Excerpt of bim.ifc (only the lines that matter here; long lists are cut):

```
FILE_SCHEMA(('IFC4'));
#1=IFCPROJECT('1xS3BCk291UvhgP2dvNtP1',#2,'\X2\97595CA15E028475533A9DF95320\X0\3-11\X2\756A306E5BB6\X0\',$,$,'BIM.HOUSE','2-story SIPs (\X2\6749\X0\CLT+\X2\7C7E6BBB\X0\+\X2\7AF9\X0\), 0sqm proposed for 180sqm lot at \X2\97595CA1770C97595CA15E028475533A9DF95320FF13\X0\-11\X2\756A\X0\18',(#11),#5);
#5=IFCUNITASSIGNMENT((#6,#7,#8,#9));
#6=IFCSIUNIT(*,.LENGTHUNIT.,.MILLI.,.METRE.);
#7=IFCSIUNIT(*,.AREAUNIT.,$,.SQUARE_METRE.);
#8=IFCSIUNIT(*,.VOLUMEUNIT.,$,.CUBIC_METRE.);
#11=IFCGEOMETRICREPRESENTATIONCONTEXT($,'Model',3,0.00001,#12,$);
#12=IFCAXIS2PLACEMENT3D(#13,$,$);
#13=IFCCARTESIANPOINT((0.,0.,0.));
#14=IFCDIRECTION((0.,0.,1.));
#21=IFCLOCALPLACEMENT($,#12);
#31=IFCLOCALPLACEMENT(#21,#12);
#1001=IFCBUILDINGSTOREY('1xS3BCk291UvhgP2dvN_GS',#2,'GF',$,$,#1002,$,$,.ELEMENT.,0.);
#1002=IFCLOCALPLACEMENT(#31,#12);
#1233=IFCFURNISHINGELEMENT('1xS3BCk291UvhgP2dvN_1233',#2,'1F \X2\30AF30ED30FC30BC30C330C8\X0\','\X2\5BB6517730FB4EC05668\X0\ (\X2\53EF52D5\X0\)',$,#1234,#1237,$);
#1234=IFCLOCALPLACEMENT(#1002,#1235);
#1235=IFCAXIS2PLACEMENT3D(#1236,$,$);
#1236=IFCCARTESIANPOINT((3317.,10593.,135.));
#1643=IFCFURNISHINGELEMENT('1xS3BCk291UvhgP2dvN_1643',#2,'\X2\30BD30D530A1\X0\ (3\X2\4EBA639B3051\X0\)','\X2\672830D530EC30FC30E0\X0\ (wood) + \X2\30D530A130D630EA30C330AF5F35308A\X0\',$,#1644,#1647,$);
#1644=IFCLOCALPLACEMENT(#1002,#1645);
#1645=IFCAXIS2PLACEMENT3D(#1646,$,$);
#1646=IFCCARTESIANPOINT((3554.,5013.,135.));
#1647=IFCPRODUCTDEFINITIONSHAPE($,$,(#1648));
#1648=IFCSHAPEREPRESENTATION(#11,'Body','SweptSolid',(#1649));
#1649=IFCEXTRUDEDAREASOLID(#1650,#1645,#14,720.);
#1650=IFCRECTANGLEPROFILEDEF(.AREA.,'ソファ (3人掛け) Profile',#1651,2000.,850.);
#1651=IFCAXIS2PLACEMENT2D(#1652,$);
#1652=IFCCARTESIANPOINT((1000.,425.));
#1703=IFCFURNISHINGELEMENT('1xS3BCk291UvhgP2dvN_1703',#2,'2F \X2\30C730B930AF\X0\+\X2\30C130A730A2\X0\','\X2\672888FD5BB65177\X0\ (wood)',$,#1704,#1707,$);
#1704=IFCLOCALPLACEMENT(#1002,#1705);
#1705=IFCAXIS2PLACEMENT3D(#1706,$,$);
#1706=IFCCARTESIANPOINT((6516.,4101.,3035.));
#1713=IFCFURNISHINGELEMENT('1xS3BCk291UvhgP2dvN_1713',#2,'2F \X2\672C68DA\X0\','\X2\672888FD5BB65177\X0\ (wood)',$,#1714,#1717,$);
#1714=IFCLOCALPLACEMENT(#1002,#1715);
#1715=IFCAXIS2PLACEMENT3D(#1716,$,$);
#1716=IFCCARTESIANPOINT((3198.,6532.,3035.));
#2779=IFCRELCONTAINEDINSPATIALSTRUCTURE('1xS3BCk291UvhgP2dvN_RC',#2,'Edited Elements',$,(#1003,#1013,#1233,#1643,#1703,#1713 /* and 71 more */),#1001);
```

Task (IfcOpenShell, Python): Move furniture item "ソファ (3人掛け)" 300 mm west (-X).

```python
import ifcopenshell
import ifcopenshell.api.geometry
import ifcopenshell.util.placement

model = ifcopenshell.open("bim.ifc")

item = model.by_guid("1xS3BCk291UvhgP2dvN_1643")
matrix = ifcopenshell.util.placement.get_local_placement(item.ObjectPlacement)
matrix[0, 3] -= 300.0
ifcopenshell.api.geometry.edit_object_placement(model, product=item, matrix=matrix, is_si=False)

print(ifcopenshell.util.placement.get_local_placement(item.ObjectPlacement).round(3) + 0.0)

model.write("bim_edited.ifc")
```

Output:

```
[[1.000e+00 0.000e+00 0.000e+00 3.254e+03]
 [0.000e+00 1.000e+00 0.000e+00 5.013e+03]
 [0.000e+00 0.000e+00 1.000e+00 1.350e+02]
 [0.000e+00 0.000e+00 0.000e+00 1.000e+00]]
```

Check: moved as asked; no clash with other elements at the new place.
